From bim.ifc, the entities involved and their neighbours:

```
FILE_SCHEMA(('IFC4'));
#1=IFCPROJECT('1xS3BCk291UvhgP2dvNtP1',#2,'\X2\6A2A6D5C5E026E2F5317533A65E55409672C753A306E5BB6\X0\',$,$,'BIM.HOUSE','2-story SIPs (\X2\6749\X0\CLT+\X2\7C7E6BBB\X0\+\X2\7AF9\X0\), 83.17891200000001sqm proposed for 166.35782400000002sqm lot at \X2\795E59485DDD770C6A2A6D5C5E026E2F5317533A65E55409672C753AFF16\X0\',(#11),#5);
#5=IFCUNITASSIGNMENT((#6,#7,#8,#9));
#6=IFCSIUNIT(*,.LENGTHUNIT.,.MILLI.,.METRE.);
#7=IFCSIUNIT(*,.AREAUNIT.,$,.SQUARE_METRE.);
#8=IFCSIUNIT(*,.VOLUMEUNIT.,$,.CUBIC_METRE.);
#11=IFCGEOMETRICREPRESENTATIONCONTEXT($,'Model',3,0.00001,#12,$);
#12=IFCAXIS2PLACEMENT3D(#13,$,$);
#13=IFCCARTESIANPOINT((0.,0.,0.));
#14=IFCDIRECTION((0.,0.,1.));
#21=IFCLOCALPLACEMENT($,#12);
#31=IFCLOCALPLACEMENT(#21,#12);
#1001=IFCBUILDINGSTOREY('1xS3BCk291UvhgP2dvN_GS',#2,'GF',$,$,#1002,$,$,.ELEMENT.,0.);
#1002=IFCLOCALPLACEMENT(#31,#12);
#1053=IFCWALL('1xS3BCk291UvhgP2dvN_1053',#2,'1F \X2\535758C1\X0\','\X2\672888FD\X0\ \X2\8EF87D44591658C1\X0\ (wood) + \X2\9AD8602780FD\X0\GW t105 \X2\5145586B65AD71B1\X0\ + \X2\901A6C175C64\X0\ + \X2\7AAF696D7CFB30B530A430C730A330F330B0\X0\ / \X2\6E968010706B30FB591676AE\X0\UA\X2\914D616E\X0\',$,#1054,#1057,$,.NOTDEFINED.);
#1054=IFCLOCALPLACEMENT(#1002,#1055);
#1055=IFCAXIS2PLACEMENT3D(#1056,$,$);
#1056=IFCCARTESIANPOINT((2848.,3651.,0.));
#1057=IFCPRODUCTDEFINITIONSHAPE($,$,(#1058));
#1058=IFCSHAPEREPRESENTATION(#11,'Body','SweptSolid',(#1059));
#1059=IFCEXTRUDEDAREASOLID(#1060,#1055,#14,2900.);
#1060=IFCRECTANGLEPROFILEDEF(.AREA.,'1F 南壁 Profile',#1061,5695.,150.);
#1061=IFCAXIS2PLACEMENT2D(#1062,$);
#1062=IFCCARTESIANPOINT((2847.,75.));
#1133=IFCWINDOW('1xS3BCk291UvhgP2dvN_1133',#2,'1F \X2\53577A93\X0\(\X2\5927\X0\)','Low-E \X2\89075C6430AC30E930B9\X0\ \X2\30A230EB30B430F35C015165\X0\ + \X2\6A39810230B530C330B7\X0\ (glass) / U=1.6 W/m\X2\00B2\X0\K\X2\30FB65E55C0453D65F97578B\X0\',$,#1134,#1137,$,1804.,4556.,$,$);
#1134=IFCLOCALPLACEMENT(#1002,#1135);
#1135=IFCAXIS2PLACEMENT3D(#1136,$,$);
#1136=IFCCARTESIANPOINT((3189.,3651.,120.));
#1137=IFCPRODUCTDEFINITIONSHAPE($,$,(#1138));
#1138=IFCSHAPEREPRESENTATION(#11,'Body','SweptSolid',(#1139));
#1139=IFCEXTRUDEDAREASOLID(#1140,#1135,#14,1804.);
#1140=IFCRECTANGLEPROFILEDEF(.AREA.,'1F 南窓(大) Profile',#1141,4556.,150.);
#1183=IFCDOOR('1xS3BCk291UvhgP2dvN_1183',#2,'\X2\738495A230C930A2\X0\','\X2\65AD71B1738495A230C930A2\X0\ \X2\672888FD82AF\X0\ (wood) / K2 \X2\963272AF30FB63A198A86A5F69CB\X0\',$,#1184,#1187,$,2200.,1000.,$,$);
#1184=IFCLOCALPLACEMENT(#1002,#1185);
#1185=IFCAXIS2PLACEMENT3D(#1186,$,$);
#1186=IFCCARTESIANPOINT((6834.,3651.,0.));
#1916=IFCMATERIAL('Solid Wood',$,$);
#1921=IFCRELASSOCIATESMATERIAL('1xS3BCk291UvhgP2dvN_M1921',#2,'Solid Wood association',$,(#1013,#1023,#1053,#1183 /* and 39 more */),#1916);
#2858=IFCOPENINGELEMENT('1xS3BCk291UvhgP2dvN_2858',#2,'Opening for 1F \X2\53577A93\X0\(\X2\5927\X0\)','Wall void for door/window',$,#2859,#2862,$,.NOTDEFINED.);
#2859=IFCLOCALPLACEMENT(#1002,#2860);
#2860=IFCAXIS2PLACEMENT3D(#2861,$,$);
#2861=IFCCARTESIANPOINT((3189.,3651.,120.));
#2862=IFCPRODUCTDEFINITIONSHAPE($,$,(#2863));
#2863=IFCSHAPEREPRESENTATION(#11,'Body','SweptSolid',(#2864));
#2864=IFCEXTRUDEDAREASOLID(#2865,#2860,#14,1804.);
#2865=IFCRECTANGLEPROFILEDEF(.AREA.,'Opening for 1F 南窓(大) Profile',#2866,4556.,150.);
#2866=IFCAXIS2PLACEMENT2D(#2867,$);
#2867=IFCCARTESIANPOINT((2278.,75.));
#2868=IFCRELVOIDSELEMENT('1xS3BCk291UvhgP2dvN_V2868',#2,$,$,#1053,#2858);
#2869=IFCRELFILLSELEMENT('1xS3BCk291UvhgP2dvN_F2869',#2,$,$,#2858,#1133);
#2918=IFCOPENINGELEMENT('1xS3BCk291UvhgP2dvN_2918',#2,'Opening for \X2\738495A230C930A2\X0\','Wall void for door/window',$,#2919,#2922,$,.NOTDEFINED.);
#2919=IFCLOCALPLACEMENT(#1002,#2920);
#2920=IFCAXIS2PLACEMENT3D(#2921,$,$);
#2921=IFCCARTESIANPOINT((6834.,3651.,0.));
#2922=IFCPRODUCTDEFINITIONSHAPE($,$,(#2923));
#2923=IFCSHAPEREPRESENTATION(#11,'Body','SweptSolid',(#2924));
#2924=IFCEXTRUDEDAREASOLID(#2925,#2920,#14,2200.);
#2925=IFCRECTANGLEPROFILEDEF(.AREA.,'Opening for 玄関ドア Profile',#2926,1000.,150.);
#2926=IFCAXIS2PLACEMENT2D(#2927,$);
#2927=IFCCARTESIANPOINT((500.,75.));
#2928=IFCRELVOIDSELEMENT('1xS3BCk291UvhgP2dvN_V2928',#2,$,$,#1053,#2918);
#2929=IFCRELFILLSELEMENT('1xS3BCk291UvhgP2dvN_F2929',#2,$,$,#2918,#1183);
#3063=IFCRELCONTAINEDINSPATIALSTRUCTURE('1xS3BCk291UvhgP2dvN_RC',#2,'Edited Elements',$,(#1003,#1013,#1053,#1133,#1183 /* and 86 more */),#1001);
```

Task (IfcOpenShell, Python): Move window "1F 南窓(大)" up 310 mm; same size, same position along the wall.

```python
import numpy as np
import ifcopenshell
import ifcopenshell.api.geometry
import ifcopenshell.util.placement
import ifcopenshell.util.unit

model = ifcopenshell.open("bim.ifc")
unit_scale = ifcopenshell.util.unit.calculate_unit_scale(model)

window = model.by_guid("1xS3BCk291UvhgP2dvN_1133")
opening = window.FillsVoids[0].RelatingOpeningElement
dz = 0.31 / unit_scale

shift = np.array([0.0, 0.0, dz])
# The window is not placed relative to its opening, so move both.
for product in (opening, window):
    matrix = ifcopenshell.util.placement.get_local_placement(product.ObjectPlacement)
    matrix[:3, 3] += shift
    ifcopenshell.api.geometry.edit_object_placement(model, product=product, matrix=matrix, is_si=False)

print(f"moved by {dz * unit_scale:+.3f} m")

model.write("bim_rev.ifc")
```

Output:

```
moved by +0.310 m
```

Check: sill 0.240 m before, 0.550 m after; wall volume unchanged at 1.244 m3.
